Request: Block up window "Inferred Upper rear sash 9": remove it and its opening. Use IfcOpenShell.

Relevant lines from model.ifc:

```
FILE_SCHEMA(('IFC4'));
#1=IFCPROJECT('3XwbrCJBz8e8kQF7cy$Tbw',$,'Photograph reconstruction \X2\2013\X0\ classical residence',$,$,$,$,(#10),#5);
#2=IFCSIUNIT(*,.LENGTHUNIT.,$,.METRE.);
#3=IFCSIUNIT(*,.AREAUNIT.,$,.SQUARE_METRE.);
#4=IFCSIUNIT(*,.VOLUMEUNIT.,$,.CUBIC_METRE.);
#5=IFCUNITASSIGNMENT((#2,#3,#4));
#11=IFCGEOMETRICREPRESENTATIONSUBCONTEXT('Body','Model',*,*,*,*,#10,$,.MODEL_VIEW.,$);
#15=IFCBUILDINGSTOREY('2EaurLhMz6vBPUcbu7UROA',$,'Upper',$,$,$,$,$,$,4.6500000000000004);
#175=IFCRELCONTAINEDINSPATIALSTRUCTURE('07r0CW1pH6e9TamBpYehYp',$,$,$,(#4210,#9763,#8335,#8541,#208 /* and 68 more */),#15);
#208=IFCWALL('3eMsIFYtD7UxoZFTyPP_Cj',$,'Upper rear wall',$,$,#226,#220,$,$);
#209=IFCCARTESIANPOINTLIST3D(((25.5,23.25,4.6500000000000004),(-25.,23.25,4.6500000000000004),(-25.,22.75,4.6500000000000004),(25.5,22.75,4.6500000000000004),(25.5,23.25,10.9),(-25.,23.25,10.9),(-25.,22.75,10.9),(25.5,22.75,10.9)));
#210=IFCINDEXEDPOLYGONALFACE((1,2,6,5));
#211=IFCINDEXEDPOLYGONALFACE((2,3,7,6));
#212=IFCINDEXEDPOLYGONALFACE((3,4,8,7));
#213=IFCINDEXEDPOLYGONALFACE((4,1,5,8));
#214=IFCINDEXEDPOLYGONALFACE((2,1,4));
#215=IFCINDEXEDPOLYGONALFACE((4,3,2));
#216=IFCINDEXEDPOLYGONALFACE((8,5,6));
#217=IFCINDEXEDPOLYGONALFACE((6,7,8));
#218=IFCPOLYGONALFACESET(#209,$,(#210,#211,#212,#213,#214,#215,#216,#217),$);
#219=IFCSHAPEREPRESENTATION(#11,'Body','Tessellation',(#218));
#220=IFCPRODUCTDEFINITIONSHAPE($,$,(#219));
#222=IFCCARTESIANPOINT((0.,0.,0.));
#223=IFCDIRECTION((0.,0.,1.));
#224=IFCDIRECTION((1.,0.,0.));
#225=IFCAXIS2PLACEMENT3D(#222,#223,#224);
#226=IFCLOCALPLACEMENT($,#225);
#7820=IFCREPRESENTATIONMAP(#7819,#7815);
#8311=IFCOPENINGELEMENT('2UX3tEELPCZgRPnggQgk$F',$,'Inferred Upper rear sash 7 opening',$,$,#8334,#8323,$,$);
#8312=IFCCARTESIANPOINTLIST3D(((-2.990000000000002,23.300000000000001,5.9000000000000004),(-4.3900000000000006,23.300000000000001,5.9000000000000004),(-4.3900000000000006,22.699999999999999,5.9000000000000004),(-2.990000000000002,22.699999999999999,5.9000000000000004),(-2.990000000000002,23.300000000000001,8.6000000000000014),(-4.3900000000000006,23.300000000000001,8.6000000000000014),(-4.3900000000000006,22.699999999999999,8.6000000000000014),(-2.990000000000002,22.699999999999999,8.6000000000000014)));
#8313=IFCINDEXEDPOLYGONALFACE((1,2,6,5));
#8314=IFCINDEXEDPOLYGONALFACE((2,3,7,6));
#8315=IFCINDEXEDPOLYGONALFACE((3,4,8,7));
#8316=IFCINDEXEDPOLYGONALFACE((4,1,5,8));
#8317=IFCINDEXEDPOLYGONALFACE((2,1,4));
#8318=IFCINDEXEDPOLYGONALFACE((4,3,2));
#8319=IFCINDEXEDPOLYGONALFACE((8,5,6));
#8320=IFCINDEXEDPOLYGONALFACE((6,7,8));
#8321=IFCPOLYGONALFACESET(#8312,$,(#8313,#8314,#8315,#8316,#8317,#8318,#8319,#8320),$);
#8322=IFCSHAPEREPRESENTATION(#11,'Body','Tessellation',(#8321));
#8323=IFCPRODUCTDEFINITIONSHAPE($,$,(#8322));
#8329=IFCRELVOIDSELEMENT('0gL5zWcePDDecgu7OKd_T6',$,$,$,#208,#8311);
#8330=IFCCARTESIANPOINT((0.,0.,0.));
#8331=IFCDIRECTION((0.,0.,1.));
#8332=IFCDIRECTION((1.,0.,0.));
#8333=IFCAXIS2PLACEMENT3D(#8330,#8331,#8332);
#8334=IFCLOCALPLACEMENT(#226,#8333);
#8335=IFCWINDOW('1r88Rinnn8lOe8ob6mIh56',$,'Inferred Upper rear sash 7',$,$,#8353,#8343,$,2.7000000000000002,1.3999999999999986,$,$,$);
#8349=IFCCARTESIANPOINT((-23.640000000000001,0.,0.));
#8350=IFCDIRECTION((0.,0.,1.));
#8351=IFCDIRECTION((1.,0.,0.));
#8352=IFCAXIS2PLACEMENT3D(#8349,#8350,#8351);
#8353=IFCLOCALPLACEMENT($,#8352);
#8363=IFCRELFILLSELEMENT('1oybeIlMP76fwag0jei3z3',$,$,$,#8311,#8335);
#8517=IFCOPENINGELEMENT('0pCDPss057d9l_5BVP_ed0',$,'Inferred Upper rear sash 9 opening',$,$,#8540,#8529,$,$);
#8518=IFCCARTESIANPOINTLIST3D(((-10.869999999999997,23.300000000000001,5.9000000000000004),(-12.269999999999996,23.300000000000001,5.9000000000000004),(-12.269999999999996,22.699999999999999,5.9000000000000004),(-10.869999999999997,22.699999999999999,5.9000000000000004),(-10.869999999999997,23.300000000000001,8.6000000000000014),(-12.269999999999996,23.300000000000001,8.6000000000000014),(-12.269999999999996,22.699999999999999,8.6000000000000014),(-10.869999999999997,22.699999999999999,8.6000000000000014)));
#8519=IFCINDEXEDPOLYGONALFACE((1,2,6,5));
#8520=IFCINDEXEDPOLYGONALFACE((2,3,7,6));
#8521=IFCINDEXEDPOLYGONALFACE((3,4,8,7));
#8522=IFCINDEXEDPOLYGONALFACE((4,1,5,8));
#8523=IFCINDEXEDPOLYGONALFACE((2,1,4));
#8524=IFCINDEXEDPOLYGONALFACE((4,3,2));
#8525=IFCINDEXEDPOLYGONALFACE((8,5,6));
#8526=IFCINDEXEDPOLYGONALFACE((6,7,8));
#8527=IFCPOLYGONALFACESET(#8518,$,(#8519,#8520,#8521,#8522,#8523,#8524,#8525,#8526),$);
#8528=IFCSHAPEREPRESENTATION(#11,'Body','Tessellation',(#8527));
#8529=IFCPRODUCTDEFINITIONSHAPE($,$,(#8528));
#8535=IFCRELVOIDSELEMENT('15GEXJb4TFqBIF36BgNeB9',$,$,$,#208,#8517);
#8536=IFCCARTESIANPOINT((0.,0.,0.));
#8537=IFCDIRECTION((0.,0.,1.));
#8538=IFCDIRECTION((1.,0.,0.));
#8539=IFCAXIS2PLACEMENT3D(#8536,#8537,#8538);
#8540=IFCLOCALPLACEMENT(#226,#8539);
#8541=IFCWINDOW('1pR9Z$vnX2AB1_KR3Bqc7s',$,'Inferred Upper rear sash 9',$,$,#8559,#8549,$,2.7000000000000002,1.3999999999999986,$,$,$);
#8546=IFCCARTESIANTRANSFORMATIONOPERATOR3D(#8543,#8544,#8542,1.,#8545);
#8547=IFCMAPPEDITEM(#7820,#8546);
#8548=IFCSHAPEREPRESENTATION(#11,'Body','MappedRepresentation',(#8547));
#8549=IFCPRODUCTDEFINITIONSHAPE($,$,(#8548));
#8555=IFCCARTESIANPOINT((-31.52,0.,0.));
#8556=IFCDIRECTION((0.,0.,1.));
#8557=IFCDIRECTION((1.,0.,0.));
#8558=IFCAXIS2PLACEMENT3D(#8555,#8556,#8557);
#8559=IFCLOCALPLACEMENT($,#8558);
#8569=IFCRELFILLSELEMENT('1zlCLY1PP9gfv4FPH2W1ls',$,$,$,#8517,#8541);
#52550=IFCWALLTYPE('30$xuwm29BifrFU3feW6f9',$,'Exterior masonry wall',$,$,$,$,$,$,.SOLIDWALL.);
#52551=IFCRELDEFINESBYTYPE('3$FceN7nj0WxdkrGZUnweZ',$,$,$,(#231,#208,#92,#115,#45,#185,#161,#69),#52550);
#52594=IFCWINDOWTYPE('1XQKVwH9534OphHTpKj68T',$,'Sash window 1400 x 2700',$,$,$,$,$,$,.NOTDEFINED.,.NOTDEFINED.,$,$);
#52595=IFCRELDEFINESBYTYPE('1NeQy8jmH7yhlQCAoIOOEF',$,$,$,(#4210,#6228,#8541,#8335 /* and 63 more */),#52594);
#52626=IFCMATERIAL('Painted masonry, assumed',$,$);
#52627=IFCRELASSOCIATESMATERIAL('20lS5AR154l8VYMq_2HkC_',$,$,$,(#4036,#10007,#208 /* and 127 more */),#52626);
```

```python
import ifcopenshell
import ifcopenshell.api.feature
import ifcopenshell.api.root
import ifcopenshell.geom
import ifcopenshell.util.shape

model = ifcopenshell.open("model.ifc")
settings = ifcopenshell.geom.settings()


def volume(element):
    """Net volume in cubic metres, openings subtracted."""
    shape = ifcopenshell.geom.create_shape(settings, element)
    return ifcopenshell.util.shape.get_volume(shape.geometry)


window = model.by_guid("1pR9Z$vnX2AB1_KR3Bqc7s")
opening = window.FillsVoids[0].RelatingOpeningElement
wall = opening.VoidsElements[0].RelatingBuildingElement
before = volume(wall)

ifcopenshell.api.root.remove_product(model, product=window)
ifcopenshell.api.feature.remove_feature(model, feature=opening)

after = volume(wall)

print(f"wall volume {before:.3f} -> {after:.3f} m3")

model.write("model_v2.ifc")
```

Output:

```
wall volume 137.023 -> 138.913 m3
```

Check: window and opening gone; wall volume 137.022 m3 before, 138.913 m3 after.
